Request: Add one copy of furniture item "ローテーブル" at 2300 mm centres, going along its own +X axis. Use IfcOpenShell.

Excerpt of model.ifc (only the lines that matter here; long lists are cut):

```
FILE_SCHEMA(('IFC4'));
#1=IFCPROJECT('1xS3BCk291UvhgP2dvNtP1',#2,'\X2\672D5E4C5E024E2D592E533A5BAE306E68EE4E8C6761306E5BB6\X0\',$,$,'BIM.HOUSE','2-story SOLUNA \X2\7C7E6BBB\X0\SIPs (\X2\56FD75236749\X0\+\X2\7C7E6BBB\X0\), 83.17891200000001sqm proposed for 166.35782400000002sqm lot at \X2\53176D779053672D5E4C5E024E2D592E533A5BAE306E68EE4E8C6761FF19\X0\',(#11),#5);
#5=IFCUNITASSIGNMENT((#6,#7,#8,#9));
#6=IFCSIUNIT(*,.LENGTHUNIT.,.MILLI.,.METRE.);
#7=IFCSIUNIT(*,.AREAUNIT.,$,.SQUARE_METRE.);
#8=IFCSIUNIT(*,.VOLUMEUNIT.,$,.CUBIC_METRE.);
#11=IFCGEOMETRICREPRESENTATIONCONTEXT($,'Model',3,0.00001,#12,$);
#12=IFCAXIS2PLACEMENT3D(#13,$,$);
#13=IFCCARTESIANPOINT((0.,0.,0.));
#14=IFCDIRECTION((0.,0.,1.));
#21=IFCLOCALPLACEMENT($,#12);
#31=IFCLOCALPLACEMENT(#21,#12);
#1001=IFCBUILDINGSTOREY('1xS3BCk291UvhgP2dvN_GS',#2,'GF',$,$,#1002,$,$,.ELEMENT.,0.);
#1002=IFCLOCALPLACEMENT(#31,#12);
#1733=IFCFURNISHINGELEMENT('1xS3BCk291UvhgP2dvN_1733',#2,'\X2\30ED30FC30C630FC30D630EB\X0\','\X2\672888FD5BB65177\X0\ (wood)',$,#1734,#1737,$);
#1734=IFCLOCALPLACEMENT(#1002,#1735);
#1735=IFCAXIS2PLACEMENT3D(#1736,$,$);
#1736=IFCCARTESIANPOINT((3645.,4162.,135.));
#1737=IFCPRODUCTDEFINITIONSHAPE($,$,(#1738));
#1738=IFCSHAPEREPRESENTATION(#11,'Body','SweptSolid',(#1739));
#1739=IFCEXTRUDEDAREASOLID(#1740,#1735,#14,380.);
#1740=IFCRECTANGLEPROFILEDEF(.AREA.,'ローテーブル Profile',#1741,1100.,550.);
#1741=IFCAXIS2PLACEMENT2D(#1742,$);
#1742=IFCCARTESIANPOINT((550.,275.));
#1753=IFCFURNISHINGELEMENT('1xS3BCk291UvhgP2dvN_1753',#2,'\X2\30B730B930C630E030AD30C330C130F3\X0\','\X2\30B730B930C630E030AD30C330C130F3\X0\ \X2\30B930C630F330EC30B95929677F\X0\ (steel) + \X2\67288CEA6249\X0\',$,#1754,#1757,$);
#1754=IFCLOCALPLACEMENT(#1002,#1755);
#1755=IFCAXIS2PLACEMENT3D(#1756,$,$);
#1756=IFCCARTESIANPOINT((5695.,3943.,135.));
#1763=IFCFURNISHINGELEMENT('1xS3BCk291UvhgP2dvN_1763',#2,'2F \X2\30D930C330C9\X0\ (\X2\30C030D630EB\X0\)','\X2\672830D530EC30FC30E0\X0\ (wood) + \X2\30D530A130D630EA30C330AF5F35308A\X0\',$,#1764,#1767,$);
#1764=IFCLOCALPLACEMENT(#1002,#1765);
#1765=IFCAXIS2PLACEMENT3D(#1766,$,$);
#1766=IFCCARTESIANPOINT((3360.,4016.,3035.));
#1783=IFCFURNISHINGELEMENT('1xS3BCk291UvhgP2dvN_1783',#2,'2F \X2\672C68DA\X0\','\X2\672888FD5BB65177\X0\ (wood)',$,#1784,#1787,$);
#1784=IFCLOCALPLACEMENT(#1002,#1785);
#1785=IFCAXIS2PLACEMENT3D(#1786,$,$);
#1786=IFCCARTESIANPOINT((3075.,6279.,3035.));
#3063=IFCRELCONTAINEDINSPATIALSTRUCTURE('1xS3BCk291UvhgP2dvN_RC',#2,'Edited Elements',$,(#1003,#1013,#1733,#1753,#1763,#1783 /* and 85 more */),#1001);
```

```python
import ifcopenshell
import ifcopenshell.api.geometry
import ifcopenshell.api.root
import ifcopenshell.util.element
import ifcopenshell.util.placement
import ifcopenshell.util.unit

model = ifcopenshell.open("model.ifc")
unit_scale = ifcopenshell.util.unit.calculate_unit_scale(model)


def reuse_history(source, copy):
    """copy_class also copies each property set's owner history, people and application; keep the originals."""
    for rel in copy.IsDefinedBy:
        if rel.is_a("IfcRelDefinesByProperties") and (history := rel.RelatingPropertyDefinition.OwnerHistory):
            rel.RelatingPropertyDefinition.OwnerHistory = source.OwnerHistory
            ifcopenshell.util.element.remove_deep2(model, history)


source = model.by_guid("1xS3BCk291UvhgP2dvN_1733")
base = ifcopenshell.util.placement.get_local_placement(source.ObjectPlacement)
step = base[:3, 0] * 2.3 / unit_scale

for i in range(1, 2):
    copy = ifcopenshell.api.root.copy_class(model, product=source)
    copy.Representation = ifcopenshell.util.element.copy_deep(
        model, source.Representation, exclude=["IfcGeometricRepresentationContext", "IfcRepresentationMap"]
    )
    reuse_history(source, copy)
    matrix = base.copy()
    matrix[:3, 3] += i * step
    print("added at", matrix[:3, 3].round(3) + 0.0)
    ifcopenshell.api.geometry.edit_object_placement(model, product=copy, matrix=matrix, is_si=False)

model.write("model_edited.ifc")
```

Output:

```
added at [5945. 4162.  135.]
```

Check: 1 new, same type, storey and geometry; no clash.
